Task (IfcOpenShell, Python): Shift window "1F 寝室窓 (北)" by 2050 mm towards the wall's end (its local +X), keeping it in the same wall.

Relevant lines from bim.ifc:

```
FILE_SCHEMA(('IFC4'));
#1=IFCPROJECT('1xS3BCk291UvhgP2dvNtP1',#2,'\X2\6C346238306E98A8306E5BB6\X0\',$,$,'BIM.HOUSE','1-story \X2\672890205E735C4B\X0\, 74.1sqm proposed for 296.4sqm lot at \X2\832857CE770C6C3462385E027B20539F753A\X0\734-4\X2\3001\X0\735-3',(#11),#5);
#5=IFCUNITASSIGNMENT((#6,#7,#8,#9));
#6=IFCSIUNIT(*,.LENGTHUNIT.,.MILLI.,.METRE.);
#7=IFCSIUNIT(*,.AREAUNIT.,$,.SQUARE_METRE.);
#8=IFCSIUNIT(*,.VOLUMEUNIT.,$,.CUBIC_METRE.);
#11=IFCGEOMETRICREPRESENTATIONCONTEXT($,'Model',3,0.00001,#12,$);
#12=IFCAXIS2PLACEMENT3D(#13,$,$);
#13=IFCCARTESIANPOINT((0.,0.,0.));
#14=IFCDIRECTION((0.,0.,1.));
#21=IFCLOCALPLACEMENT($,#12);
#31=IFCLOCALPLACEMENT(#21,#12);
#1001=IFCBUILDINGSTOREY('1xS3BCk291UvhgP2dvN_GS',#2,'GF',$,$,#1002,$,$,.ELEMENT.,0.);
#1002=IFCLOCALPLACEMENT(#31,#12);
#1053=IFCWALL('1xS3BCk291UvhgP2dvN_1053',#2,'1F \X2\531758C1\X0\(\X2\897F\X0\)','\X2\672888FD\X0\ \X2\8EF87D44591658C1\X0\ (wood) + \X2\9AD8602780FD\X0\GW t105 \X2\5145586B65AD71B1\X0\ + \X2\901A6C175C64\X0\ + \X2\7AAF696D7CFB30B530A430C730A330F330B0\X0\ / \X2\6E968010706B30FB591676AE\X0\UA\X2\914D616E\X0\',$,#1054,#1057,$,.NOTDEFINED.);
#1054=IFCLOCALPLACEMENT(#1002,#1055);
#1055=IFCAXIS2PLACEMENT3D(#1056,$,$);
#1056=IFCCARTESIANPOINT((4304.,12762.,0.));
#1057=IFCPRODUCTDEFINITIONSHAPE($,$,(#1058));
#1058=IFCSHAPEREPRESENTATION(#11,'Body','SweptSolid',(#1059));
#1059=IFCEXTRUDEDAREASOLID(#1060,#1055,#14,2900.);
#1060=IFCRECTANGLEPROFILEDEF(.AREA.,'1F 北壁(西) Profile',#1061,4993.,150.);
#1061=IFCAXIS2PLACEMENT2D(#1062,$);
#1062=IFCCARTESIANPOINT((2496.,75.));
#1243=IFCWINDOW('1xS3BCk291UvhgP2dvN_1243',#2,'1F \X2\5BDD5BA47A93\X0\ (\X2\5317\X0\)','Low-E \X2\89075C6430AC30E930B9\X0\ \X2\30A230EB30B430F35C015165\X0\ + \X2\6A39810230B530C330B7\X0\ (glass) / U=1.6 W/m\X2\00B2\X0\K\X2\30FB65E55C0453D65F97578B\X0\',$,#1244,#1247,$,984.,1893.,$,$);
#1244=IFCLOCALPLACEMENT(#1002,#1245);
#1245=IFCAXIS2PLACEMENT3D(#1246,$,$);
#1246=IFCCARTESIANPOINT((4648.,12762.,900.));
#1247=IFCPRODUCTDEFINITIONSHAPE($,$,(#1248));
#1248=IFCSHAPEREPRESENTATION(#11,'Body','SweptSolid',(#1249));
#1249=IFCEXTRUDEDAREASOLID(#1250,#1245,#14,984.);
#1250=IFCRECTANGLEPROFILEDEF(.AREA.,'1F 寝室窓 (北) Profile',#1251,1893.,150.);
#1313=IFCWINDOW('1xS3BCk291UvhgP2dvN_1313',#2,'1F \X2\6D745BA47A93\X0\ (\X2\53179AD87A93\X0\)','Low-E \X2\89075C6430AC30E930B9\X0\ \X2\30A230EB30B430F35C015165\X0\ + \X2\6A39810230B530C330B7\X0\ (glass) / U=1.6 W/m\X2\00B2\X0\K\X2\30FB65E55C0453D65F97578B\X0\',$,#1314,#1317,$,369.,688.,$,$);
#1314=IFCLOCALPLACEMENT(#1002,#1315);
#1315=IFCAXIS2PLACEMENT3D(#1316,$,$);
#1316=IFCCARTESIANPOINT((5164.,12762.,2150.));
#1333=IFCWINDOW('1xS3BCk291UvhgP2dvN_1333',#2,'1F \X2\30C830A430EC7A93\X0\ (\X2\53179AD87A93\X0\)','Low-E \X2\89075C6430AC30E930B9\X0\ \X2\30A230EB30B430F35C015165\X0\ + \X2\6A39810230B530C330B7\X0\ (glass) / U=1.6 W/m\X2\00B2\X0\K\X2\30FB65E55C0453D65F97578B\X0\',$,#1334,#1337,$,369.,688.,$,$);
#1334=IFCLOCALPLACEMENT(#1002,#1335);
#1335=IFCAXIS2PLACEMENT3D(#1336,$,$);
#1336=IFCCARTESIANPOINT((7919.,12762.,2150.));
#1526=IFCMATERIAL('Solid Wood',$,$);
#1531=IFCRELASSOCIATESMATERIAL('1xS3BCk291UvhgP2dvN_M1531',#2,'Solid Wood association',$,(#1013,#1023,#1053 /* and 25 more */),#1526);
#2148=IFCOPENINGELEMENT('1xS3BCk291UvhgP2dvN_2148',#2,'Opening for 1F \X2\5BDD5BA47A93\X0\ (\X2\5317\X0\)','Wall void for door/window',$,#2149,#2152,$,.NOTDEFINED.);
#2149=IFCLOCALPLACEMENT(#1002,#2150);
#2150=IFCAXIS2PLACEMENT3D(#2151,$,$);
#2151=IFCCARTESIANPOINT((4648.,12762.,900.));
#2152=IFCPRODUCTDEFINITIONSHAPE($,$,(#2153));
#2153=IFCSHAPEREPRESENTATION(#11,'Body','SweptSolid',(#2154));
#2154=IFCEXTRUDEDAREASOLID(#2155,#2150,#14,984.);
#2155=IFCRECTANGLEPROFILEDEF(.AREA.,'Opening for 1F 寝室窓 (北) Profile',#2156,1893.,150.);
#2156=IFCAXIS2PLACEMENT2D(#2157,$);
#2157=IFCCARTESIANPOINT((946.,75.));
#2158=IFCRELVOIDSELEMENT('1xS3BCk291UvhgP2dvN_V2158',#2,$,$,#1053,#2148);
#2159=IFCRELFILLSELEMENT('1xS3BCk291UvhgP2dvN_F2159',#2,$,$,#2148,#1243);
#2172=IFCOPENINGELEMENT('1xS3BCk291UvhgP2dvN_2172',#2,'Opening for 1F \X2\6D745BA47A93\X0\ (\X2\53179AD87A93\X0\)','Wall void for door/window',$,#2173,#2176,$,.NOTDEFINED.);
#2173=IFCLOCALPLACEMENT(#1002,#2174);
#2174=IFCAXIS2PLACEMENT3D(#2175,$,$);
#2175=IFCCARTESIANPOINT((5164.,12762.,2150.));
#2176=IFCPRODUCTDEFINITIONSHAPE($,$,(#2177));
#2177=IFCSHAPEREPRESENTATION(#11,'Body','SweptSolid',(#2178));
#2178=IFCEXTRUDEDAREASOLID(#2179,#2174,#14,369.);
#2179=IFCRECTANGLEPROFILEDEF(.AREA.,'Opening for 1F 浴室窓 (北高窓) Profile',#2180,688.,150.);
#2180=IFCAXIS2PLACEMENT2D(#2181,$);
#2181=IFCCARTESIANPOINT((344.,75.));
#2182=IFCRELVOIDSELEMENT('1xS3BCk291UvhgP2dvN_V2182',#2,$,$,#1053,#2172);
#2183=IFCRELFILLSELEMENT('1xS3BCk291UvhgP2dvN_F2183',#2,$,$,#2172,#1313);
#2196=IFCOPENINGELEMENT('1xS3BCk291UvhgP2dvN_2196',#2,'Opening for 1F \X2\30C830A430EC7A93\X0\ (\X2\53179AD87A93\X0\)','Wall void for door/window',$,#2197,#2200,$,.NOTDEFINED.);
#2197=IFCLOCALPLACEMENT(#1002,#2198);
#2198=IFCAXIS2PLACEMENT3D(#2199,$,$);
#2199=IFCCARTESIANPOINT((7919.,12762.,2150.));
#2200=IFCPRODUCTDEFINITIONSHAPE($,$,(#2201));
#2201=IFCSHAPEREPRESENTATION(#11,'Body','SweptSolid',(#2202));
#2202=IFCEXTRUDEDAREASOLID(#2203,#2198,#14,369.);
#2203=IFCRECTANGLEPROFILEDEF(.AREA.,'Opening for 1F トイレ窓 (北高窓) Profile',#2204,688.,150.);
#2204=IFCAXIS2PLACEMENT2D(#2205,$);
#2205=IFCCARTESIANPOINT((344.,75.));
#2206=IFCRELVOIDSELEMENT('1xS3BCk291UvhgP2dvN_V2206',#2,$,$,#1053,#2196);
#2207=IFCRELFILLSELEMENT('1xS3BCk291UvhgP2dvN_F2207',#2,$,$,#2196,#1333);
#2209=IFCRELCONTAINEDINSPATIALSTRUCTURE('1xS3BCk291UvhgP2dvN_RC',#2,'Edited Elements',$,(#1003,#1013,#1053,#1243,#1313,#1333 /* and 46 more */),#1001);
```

```python
import ifcopenshell
import ifcopenshell.api.geometry
import ifcopenshell.util.placement
import ifcopenshell.util.unit

model = ifcopenshell.open("bim.ifc")
unit_scale = ifcopenshell.util.unit.calculate_unit_scale(model)

window = model.by_guid("1xS3BCk291UvhgP2dvN_1243")
opening = window.FillsVoids[0].RelatingOpeningElement
wall = opening.VoidsElements[0].RelatingBuildingElement

wall_matrix = ifcopenshell.util.placement.get_local_placement(wall.ObjectPlacement)
shift = wall_matrix[:3, 0] * 2.05 / unit_scale
before = ifcopenshell.util.placement.get_local_placement(window.ObjectPlacement)[:3, 3].copy()

# The window is not placed relative to its opening, so move both.
for product in (opening, window):
    matrix = ifcopenshell.util.placement.get_local_placement(product.ObjectPlacement)
    matrix[:3, 3] += shift
    ifcopenshell.api.geometry.edit_object_placement(model, product=product, matrix=matrix, is_si=False)

after = ifcopenshell.util.placement.get_local_placement(window.ObjectPlacement)[:3, 3]
print("window moved by", (after - before).round(3) + 0.0)

model.write("bim_updated.ifc")
```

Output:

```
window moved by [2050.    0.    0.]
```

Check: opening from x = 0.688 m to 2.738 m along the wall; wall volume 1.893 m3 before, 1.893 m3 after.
